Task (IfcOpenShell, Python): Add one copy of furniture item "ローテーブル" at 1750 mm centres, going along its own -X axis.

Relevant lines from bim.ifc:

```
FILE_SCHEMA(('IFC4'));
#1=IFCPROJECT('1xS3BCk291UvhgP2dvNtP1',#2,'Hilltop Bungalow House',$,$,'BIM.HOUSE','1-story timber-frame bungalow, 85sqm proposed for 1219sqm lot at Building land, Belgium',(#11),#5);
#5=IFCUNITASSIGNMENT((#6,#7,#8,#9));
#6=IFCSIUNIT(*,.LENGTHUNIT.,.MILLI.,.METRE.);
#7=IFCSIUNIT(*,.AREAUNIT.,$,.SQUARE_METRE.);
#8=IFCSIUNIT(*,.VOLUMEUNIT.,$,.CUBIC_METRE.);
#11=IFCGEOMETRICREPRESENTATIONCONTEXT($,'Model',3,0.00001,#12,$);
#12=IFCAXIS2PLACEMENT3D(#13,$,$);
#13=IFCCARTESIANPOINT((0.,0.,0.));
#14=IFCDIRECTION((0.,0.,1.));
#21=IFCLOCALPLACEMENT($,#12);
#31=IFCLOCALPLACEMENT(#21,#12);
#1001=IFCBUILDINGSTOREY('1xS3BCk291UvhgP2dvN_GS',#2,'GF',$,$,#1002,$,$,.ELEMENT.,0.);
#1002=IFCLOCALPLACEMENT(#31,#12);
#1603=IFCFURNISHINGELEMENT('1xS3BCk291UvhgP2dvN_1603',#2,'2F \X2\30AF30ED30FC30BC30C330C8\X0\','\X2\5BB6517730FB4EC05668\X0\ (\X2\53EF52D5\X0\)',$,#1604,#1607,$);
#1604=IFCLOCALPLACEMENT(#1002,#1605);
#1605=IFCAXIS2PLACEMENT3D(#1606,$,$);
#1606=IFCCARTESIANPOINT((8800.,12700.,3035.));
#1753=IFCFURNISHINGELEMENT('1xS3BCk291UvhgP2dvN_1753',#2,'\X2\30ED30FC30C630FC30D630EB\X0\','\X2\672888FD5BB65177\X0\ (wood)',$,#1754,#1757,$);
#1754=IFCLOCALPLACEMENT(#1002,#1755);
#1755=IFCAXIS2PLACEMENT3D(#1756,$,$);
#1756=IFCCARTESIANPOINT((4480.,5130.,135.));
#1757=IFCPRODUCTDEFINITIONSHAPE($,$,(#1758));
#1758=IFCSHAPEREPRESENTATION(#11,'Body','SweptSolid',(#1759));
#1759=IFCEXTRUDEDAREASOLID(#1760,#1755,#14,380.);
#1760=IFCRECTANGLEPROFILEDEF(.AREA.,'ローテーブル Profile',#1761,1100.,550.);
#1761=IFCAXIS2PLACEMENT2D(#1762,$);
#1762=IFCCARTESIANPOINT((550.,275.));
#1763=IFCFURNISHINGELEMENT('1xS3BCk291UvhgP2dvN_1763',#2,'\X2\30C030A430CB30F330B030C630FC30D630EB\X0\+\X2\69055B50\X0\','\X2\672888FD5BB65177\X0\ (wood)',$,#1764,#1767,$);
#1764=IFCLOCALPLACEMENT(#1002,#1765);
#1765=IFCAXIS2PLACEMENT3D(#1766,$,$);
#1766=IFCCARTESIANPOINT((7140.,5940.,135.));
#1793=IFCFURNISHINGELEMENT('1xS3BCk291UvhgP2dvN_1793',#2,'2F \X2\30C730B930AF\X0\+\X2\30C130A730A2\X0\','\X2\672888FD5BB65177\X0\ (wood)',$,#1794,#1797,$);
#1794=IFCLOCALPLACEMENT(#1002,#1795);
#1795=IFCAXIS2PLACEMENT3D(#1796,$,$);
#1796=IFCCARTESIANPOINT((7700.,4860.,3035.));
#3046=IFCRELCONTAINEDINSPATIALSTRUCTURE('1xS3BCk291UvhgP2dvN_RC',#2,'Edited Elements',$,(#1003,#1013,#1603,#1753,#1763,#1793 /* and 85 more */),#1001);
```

```python
import ifcopenshell
import ifcopenshell.api.geometry
import ifcopenshell.api.root
import ifcopenshell.util.element
import ifcopenshell.util.placement
import ifcopenshell.util.unit

model = ifcopenshell.open("bim.ifc")
unit_scale = ifcopenshell.util.unit.calculate_unit_scale(model)


def reuse_history(source, copy):
    """copy_class also copies each property set's owner history, people and application; keep the originals."""
    for rel in copy.IsDefinedBy:
        if rel.is_a("IfcRelDefinesByProperties") and (history := rel.RelatingPropertyDefinition.OwnerHistory):
            rel.RelatingPropertyDefinition.OwnerHistory = source.OwnerHistory
            ifcopenshell.util.element.remove_deep2(model, history)


source = model.by_guid("1xS3BCk291UvhgP2dvN_1753")
base = ifcopenshell.util.placement.get_local_placement(source.ObjectPlacement)
step = -base[:3, 0] * 1.75 / unit_scale

for i in range(1, 2):
    copy = ifcopenshell.api.root.copy_class(model, product=source)
    copy.Representation = ifcopenshell.util.element.copy_deep(
        model, source.Representation, exclude=["IfcGeometricRepresentationContext", "IfcRepresentationMap"]
    )
    reuse_history(source, copy)
    matrix = base.copy()
    matrix[:3, 3] += i * step
    print("added at", matrix[:3, 3].round(3) + 0.0)
    ifcopenshell.api.geometry.edit_object_placement(model, product=copy, matrix=matrix, is_si=False)

model.write("bim_v2.ifc")
```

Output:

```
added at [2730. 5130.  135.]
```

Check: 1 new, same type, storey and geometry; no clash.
